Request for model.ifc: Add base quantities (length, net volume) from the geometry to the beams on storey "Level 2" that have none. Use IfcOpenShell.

First a look at what the model holds.

```python
import ifcopenshell
import ifcopenshell.util.element
import ifcopenshell.util.unit

model = ifcopenshell.open("model.ifc")
print(model.schema)
for unit_type in ("LENGTHUNIT", "AREAUNIT", "VOLUMEUNIT"):
    print(unit_type, ifcopenshell.util.unit.calculate_unit_scale(model, unit_type))
storey = next(s for s in model.by_type("IfcBuildingStorey") if s.Name == "Level 2")
beams = [e for e in ifcopenshell.util.element.get_decomposition(storey) if e.is_a("IfcBeam")]
for e in sorted(beams, key=lambda e: e.id()):
    print(e.id(), e.is_a(), e.Name, list(ifcopenshell.util.element.get_psets(e, qtos_only=True)), sep=" | ")
```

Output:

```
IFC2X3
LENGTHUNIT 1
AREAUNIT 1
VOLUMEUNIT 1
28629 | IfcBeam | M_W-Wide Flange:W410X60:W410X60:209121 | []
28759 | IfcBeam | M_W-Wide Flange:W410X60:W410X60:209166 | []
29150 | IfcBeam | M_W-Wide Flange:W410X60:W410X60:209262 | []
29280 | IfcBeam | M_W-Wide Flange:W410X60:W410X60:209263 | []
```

```python
import ifcopenshell
import ifcopenshell.api.pset
import ifcopenshell.geom
import ifcopenshell.util.element
import ifcopenshell.util.shape
import ifcopenshell.util.unit

model = ifcopenshell.open("model.ifc")
unit_scale = ifcopenshell.util.unit.calculate_unit_scale(model)
volume_scale = ifcopenshell.util.unit.calculate_unit_scale(model, "VOLUMEUNIT")
settings = ifcopenshell.geom.settings()

storey = next(s for s in model.by_type("IfcBuildingStorey") if s.Name == "Level 2")
beams = [e for e in ifcopenshell.util.element.get_decomposition(storey) if e.is_a("IfcBeam")]

for e in sorted(beams, key=lambda e: e.id()):
    if ifcopenshell.util.element.get_psets(e, qtos_only=True, should_inherit=False):
        continue
    # Geometry comes back in metres, in the element's own axes.
    shape = ifcopenshell.geom.create_shape(settings, e)
    values = {
        "Length": ifcopenshell.util.shape.get_max_xyz(shape.geometry) / unit_scale,
        "NetVolume": ifcopenshell.util.shape.get_volume(shape.geometry) / volume_scale,
    }
    qto = ifcopenshell.api.pset.add_qto(model, product=e, name="BaseQuantities")
    ifcopenshell.api.pset.edit_qto(model, qto=qto, properties=values)
    print(e.id(), {k: round(v, 3) for k, v in values.items()})

model.write("model_updated.ifc")
```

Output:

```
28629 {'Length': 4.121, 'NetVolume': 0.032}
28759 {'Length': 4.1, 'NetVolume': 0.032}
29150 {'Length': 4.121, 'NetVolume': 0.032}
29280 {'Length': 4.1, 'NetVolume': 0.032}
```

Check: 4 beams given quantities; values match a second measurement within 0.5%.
